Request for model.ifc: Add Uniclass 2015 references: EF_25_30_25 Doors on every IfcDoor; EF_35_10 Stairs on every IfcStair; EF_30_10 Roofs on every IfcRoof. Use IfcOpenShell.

First a look at what the model holds.

```python
import ifcopenshell

model = ifcopenshell.open("model.ifc")
print(model.schema)
print("classifications:", [c.Name for c in model.by_type("IfcClassification")])
for ifc_class in ("IfcDoor", "IfcRoof", "IfcStair", "IfcWall", "IfcWindow"):
    print(ifc_class, len(model.by_type(ifc_class)))
```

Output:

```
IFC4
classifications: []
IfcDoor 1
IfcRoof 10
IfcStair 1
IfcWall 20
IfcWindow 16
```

```python
import ifcopenshell
import ifcopenshell.api.classification

model = ifcopenshell.open("model.ifc")

system = ifcopenshell.api.classification.add_classification(model, classification="Uniclass 2015")

codes = {
    "IfcDoor": ("EF_25_30_25", "Doors"),
    "IfcStair": ("EF_35_10", "Stairs"),
    "IfcRoof": ("EF_30_10", "Roofs"),
}
for ifc_class, (code, name) in codes.items():
    products = model.by_type(ifc_class)
    ifcopenshell.api.classification.add_reference(
        model, products=products, classification=system, identification=code, name=name
    )
    print(code, len(products))

model.write("model_updated.ifc")
```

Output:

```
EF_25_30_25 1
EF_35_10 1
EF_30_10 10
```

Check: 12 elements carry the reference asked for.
